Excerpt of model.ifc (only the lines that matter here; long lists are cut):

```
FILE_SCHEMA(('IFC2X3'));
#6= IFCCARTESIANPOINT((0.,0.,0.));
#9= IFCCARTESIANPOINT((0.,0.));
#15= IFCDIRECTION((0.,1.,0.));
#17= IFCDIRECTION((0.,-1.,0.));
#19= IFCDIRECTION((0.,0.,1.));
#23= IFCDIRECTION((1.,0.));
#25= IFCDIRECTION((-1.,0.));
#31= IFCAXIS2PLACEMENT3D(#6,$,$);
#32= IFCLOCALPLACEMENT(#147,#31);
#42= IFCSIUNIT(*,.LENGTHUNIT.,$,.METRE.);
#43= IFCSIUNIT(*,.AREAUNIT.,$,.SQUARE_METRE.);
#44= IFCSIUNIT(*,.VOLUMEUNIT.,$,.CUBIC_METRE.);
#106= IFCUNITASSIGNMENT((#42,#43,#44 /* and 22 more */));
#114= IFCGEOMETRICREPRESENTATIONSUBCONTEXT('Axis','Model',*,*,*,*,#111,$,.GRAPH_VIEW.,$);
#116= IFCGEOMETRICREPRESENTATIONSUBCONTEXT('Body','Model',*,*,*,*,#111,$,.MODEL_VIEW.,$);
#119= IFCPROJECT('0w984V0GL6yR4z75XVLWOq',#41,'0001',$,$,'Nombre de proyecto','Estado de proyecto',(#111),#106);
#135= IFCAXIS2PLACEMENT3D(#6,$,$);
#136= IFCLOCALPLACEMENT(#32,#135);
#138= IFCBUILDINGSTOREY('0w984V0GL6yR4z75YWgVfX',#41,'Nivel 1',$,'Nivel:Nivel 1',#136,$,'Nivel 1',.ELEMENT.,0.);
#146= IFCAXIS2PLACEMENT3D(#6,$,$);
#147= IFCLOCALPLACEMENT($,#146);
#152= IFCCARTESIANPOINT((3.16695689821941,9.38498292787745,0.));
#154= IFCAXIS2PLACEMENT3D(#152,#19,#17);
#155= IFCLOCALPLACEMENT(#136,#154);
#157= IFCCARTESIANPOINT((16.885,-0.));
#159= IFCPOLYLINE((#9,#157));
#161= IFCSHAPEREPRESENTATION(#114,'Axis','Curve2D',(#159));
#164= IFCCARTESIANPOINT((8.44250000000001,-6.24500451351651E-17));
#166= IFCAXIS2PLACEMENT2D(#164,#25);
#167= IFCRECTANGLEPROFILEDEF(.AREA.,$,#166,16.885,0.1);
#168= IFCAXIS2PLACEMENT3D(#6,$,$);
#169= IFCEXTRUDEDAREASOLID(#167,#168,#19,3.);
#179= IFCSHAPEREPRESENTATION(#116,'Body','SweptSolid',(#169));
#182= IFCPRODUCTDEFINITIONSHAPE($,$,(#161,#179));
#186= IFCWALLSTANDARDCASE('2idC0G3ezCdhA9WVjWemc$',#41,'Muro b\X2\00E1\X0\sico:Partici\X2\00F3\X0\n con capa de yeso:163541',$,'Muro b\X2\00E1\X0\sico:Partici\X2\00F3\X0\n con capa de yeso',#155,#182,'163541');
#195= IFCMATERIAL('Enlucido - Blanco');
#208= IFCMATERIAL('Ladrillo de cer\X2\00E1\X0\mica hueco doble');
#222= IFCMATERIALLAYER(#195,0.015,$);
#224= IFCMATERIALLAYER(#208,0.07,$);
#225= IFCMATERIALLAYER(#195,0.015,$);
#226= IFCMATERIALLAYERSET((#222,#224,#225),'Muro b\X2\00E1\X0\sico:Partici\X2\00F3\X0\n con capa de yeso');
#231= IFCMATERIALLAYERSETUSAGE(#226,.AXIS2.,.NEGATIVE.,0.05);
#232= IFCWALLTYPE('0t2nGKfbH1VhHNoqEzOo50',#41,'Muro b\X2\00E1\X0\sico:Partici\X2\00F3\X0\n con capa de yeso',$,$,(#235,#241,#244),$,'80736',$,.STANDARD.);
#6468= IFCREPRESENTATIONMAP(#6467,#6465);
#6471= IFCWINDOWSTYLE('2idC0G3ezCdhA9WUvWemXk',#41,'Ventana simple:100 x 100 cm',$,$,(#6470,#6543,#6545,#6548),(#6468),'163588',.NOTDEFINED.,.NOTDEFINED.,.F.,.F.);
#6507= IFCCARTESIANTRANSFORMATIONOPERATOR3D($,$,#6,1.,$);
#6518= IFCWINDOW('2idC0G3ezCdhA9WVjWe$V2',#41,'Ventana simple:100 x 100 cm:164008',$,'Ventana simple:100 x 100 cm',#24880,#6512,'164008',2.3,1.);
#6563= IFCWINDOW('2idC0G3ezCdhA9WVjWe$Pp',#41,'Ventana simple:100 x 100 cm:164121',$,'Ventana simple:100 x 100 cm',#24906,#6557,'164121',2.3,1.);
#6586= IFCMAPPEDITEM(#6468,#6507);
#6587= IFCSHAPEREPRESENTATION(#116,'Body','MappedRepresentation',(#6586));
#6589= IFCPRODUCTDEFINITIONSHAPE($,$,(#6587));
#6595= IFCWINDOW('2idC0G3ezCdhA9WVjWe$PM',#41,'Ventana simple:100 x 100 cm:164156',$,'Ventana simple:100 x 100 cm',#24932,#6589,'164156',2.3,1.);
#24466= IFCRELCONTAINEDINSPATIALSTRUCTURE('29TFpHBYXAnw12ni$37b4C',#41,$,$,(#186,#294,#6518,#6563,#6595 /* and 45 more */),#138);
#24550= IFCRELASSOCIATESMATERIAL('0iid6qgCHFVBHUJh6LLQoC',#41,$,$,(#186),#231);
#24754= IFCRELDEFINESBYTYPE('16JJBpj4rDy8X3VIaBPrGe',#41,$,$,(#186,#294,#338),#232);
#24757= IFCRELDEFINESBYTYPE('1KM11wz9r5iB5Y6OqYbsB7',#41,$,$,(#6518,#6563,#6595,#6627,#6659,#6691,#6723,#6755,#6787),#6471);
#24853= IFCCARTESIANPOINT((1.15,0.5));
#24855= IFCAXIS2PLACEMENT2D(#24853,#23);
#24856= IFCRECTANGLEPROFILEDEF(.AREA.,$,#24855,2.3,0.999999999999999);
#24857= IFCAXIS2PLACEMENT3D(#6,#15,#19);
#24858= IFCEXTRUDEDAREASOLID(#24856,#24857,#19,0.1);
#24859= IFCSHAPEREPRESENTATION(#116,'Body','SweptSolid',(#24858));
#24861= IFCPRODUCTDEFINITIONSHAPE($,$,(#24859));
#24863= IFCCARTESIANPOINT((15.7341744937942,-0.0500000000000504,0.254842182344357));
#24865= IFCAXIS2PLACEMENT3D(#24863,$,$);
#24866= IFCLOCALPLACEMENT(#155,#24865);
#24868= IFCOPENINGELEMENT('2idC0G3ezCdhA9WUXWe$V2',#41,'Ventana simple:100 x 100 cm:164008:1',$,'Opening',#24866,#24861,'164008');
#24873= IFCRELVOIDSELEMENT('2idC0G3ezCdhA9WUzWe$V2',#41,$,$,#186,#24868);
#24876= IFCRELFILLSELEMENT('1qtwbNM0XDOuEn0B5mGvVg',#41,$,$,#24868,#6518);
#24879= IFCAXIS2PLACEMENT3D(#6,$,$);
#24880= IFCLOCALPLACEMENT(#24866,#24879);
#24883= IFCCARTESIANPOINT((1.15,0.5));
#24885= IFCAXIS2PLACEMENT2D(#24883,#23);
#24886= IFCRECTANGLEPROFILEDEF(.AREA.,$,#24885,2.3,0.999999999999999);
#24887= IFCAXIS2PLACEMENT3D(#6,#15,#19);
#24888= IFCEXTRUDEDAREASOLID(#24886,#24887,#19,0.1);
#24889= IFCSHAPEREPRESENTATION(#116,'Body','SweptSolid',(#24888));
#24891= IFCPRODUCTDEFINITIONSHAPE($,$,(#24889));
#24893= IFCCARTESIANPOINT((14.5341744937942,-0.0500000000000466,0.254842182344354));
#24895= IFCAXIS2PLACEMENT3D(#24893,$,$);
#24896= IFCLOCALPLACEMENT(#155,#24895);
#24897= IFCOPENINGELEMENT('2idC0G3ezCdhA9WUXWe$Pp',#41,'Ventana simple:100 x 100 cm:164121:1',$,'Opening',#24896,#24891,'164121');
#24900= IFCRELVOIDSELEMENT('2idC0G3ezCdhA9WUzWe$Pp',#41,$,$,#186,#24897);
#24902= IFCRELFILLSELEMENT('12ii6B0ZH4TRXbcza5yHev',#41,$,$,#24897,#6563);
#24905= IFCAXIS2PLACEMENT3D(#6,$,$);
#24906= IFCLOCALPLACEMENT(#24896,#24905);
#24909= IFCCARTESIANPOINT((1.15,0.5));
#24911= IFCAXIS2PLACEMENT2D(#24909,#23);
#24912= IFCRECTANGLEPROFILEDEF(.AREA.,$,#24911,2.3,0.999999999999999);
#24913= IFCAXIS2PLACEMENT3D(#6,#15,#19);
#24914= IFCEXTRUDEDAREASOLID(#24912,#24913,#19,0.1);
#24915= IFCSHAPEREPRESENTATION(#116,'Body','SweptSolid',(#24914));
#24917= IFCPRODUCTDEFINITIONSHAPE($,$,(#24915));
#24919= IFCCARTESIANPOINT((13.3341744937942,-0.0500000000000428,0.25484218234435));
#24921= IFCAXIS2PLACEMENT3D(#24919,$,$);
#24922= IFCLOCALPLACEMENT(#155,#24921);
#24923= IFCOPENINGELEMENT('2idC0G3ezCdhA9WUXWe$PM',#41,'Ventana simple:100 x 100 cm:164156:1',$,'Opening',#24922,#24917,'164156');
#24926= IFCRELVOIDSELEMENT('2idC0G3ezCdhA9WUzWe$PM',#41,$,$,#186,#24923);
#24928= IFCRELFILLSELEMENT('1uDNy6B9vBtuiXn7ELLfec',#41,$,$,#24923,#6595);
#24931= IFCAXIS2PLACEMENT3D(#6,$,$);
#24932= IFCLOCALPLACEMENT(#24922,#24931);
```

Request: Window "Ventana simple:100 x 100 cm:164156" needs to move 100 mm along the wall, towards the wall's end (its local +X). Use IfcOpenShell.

```python
import ifcopenshell
import ifcopenshell.api.geometry
import ifcopenshell.util.placement

model = ifcopenshell.open("model.ifc")

window = model.by_id(6595)
opening = window.FillsVoids[0].RelatingOpeningElement
wall = opening.VoidsElements[0].RelatingBuildingElement

wall_matrix = ifcopenshell.util.placement.get_local_placement(wall.ObjectPlacement)
shift = wall_matrix[:3, 0] * 0.1
before = ifcopenshell.util.placement.get_local_placement(window.ObjectPlacement)[:3, 3].copy()

# The window is placed relative to its opening, so it follows when the opening moves.
matrix = ifcopenshell.util.placement.get_local_placement(opening.ObjectPlacement)
matrix[:3, 3] += shift
ifcopenshell.api.geometry.edit_object_placement(
    model, product=opening, matrix=matrix, is_si=False, should_transform_children=True
)

after = ifcopenshell.util.placement.get_local_placement(window.ObjectPlacement)[:3, 3]
print("window moved by", (after - before).round(3) + 0.0)

model.write("model_v2.ifc")
```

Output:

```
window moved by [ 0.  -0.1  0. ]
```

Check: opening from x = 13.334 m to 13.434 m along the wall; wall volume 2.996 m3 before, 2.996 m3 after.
